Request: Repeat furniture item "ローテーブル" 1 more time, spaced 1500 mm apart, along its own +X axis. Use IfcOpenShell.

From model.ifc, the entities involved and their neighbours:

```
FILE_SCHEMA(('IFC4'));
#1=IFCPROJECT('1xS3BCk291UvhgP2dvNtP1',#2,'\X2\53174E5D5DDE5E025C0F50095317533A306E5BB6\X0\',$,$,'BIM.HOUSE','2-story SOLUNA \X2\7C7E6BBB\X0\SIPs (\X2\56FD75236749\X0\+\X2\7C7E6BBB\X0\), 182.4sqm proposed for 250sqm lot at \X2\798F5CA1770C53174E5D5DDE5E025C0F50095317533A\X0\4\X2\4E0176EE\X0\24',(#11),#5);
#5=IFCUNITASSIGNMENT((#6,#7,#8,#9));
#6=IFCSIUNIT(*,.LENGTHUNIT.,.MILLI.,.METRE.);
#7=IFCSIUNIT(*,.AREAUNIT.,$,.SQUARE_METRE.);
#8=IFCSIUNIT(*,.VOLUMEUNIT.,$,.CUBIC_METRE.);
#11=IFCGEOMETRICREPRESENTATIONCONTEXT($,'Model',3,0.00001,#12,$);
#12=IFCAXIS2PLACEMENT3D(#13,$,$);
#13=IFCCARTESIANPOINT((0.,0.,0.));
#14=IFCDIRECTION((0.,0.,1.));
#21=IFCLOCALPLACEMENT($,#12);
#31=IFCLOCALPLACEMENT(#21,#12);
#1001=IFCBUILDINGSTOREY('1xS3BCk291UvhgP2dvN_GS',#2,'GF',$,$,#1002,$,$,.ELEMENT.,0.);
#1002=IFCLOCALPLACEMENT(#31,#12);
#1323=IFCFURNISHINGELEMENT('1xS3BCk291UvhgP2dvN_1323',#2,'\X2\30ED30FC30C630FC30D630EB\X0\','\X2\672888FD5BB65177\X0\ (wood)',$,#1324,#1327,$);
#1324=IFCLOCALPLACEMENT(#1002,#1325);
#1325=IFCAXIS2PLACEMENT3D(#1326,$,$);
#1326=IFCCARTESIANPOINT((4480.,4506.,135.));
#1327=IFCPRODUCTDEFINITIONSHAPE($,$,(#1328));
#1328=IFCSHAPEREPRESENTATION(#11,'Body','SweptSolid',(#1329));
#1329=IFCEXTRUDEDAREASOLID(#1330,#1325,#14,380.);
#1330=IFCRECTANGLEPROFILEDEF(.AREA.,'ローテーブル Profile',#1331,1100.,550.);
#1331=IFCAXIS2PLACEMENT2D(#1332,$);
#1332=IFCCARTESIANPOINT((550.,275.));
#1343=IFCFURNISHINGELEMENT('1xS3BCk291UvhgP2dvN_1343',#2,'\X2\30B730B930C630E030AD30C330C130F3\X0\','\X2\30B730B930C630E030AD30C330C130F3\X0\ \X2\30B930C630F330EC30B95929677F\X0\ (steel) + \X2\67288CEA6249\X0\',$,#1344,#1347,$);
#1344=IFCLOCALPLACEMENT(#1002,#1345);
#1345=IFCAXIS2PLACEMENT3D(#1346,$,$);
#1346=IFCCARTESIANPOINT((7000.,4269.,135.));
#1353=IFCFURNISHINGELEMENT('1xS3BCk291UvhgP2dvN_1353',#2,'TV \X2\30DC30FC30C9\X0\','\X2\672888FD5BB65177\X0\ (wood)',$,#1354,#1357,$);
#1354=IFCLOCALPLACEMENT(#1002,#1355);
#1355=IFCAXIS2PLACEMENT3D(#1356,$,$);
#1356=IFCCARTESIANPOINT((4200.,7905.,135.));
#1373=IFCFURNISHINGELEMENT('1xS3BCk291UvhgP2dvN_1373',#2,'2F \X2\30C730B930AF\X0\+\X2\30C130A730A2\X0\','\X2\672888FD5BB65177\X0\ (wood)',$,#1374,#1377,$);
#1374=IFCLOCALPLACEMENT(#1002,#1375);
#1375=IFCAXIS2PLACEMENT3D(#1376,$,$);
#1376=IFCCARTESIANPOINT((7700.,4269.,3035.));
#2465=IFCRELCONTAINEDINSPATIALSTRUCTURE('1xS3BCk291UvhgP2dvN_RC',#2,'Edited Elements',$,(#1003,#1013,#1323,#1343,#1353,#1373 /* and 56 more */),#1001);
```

```python
import ifcopenshell
import ifcopenshell.api.geometry
import ifcopenshell.api.root
import ifcopenshell.util.element
import ifcopenshell.util.placement

model = ifcopenshell.open("model.ifc")


def reuse_history(source, copy):
    """copy_class also copies each property set's owner history, people and application; keep the originals."""
    for rel in copy.IsDefinedBy:
        if rel.is_a("IfcRelDefinesByProperties") and (history := rel.RelatingPropertyDefinition.OwnerHistory):
            rel.RelatingPropertyDefinition.OwnerHistory = source.OwnerHistory
            ifcopenshell.util.element.remove_deep2(model, history)


source = model.by_id(1323)
base = ifcopenshell.util.placement.get_local_placement(source.ObjectPlacement)
step = base[:3, 0] * 1500.0

for i in range(1, 2):
    copy = ifcopenshell.api.root.copy_class(model, product=source)
    copy.Representation = ifcopenshell.util.element.copy_deep(
        model, source.Representation, exclude=["IfcGeometricRepresentationContext", "IfcRepresentationMap"]
    )
    reuse_history(source, copy)
    matrix = base.copy()
    matrix[:3, 3] += i * step
    print("added at", matrix[:3, 3].round(3) + 0.0)
    ifcopenshell.api.geometry.edit_object_placement(model, product=copy, matrix=matrix, is_si=False)

model.write("model-out.ifc")
```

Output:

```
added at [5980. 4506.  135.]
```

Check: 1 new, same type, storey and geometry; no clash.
